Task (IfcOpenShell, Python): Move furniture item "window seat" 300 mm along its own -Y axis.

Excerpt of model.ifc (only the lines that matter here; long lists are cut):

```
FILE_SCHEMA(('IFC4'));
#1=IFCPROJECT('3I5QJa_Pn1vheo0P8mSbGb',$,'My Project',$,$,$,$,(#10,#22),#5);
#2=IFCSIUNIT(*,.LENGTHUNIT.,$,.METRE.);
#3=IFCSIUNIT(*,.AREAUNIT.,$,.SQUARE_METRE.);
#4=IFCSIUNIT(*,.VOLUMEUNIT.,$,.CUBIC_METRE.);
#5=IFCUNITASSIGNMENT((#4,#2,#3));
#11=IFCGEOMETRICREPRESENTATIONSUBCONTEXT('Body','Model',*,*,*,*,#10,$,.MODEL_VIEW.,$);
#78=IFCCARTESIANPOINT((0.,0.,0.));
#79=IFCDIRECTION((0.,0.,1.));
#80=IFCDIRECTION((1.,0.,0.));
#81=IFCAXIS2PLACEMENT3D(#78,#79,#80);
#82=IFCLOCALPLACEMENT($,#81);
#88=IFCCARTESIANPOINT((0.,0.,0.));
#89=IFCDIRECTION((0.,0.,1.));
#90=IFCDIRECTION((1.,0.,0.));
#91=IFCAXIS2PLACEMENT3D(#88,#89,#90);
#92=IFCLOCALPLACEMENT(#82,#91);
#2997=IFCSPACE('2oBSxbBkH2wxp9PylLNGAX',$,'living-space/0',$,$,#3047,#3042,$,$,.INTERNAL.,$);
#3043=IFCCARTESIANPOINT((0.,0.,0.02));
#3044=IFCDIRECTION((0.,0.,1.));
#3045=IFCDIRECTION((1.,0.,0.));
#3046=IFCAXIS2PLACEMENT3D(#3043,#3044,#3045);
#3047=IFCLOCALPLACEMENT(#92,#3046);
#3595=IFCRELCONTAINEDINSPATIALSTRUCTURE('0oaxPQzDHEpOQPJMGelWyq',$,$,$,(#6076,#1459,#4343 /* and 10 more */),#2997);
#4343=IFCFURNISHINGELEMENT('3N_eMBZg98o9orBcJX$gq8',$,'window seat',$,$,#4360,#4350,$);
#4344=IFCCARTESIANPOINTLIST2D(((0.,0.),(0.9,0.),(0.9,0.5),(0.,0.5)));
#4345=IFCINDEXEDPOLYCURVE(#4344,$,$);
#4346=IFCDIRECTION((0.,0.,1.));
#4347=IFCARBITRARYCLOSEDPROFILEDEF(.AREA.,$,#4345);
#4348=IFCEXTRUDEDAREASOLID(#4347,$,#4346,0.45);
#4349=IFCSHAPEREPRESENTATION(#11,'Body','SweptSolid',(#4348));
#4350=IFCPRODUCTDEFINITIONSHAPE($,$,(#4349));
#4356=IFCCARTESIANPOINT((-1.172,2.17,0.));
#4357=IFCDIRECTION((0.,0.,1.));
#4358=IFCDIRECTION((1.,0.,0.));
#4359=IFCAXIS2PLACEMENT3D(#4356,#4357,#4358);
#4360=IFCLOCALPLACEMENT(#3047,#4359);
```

```python
import ifcopenshell
import ifcopenshell.api.geometry
import ifcopenshell.util.placement

model = ifcopenshell.open("model.ifc")

item = model.by_guid("3N_eMBZg98o9orBcJX$gq8")
matrix = ifcopenshell.util.placement.get_local_placement(item.ObjectPlacement)
matrix[:3, 3] -= matrix[:3, 1] * 0.3
ifcopenshell.api.geometry.edit_object_placement(model, product=item, matrix=matrix, is_si=False)

print(ifcopenshell.util.placement.get_local_placement(item.ObjectPlacement).round(3) + 0.0)

model.write("model_updated.ifc")
```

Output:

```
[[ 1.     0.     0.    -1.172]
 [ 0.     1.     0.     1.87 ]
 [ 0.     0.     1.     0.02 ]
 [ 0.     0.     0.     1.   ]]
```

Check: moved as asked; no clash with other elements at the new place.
